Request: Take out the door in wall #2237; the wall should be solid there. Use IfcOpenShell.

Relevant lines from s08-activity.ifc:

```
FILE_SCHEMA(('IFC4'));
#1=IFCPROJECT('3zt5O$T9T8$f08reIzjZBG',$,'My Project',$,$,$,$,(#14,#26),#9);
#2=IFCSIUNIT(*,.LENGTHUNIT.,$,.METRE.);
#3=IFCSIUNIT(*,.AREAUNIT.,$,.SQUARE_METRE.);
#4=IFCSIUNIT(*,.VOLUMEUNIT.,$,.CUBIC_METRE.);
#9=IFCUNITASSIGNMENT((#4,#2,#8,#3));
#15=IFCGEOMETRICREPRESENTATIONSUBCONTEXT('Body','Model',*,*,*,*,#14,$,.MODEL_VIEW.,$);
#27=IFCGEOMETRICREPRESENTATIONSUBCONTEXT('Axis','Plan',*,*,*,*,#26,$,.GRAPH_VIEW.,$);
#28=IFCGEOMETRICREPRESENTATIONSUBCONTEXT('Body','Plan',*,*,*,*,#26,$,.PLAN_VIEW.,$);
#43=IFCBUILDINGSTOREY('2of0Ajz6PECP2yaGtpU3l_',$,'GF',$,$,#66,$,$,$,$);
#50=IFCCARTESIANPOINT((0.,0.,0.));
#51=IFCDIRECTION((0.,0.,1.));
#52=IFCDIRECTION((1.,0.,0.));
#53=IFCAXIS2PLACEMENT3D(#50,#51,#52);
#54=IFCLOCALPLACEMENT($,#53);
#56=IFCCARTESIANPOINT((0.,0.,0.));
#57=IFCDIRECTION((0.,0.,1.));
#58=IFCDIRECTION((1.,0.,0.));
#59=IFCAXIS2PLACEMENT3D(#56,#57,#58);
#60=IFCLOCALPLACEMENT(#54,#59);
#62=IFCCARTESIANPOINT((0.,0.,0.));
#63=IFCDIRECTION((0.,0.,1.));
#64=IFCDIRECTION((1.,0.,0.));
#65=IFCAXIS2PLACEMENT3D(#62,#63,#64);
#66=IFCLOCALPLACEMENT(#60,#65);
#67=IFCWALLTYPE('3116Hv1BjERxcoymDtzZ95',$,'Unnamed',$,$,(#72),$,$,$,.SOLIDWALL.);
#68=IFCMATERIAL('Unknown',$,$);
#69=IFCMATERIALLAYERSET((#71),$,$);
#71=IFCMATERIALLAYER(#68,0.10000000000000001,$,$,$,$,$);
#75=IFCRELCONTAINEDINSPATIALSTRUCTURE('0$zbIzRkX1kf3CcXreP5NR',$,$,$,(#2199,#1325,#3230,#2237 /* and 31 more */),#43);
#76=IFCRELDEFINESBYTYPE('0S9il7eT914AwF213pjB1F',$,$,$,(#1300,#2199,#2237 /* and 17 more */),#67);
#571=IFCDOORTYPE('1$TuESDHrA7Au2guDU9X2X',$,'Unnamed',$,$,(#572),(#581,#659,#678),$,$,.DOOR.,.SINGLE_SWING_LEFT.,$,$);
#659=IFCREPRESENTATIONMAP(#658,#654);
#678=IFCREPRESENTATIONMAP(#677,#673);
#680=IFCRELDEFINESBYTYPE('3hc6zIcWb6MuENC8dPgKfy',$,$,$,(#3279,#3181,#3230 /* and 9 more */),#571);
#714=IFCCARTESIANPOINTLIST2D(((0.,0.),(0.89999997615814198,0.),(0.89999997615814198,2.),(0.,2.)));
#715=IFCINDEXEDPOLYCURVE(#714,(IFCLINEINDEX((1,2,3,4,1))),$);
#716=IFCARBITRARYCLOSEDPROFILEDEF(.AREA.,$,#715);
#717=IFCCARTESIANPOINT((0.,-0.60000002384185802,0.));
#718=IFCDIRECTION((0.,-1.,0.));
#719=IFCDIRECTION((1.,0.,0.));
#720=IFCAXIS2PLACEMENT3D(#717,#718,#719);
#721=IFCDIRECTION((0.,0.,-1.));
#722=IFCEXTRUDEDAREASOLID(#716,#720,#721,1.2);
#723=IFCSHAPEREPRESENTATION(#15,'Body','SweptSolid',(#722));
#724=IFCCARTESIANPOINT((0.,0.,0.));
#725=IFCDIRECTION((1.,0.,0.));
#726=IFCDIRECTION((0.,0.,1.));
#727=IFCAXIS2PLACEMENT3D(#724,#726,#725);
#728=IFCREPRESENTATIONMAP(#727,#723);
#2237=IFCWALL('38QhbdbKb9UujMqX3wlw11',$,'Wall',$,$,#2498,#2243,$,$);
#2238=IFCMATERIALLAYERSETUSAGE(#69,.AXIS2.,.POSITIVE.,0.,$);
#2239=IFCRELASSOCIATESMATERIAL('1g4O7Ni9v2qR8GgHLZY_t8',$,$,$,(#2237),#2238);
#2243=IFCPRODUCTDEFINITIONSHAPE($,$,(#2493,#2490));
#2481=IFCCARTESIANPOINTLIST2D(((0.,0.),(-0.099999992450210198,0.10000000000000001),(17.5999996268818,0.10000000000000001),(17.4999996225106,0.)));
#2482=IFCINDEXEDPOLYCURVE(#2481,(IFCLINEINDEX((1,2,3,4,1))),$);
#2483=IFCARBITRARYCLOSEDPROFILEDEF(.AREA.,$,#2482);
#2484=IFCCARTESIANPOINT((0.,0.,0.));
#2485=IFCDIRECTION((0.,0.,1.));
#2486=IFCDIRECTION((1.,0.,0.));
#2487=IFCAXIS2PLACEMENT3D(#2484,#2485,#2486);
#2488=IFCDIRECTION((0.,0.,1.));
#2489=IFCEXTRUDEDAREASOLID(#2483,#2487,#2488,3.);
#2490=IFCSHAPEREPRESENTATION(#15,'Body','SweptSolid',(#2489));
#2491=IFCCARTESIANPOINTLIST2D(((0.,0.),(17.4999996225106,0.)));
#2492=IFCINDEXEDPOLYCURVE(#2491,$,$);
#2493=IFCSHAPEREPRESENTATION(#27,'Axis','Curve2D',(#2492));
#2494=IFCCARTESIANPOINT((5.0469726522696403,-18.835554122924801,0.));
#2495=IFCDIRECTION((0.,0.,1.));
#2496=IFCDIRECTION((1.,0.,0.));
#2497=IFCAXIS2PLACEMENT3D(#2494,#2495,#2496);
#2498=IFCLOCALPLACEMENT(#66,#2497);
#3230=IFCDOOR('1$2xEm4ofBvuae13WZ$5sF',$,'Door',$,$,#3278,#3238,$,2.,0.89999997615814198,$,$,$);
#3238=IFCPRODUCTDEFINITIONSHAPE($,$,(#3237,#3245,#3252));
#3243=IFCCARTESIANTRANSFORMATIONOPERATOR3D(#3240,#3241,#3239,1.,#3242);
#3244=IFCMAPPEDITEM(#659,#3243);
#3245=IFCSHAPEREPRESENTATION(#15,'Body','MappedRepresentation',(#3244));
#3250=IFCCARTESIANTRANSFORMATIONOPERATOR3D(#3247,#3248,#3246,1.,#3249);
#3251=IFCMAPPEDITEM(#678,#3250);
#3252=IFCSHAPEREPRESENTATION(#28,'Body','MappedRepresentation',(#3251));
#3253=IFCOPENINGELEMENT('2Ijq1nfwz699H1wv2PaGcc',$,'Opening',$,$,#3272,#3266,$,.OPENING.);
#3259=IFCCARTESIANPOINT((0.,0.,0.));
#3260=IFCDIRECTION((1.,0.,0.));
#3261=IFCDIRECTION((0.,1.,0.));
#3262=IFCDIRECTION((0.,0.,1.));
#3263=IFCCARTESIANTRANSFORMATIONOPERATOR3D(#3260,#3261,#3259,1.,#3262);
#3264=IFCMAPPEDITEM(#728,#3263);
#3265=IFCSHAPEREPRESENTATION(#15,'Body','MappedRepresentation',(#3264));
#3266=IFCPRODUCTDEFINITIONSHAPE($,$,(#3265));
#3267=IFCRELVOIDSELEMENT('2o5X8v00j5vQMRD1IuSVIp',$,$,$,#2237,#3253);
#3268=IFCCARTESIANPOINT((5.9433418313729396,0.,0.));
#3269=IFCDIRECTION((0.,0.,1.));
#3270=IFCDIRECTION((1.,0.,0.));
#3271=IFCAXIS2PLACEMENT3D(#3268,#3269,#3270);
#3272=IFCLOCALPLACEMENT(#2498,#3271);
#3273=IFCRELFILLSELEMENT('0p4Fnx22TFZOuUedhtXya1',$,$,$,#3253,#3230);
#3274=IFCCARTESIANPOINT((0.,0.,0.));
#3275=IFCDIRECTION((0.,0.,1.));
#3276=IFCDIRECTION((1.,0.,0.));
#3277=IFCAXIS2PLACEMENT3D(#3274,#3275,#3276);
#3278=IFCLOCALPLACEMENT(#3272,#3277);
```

```python
import ifcopenshell
import ifcopenshell.api.feature
import ifcopenshell.api.root
import ifcopenshell.geom
import ifcopenshell.util.shape

model = ifcopenshell.open("s08-activity.ifc")
settings = ifcopenshell.geom.settings()


def volume(element):
    """Net volume in cubic metres, openings subtracted."""
    shape = ifcopenshell.geom.create_shape(settings, element)
    return ifcopenshell.util.shape.get_volume(shape.geometry)


door = model.by_id(3230)
opening = door.FillsVoids[0].RelatingOpeningElement
wall = opening.VoidsElements[0].RelatingBuildingElement
before = volume(wall)

ifcopenshell.api.root.remove_product(model, product=door)
ifcopenshell.api.feature.remove_feature(model, feature=opening)

after = volume(wall)

print(f"wall volume {before:.3f} -> {after:.3f} m3")

model.write("s08-activity_updated.ifc")
```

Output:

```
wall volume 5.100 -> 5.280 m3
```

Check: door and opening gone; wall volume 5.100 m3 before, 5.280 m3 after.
